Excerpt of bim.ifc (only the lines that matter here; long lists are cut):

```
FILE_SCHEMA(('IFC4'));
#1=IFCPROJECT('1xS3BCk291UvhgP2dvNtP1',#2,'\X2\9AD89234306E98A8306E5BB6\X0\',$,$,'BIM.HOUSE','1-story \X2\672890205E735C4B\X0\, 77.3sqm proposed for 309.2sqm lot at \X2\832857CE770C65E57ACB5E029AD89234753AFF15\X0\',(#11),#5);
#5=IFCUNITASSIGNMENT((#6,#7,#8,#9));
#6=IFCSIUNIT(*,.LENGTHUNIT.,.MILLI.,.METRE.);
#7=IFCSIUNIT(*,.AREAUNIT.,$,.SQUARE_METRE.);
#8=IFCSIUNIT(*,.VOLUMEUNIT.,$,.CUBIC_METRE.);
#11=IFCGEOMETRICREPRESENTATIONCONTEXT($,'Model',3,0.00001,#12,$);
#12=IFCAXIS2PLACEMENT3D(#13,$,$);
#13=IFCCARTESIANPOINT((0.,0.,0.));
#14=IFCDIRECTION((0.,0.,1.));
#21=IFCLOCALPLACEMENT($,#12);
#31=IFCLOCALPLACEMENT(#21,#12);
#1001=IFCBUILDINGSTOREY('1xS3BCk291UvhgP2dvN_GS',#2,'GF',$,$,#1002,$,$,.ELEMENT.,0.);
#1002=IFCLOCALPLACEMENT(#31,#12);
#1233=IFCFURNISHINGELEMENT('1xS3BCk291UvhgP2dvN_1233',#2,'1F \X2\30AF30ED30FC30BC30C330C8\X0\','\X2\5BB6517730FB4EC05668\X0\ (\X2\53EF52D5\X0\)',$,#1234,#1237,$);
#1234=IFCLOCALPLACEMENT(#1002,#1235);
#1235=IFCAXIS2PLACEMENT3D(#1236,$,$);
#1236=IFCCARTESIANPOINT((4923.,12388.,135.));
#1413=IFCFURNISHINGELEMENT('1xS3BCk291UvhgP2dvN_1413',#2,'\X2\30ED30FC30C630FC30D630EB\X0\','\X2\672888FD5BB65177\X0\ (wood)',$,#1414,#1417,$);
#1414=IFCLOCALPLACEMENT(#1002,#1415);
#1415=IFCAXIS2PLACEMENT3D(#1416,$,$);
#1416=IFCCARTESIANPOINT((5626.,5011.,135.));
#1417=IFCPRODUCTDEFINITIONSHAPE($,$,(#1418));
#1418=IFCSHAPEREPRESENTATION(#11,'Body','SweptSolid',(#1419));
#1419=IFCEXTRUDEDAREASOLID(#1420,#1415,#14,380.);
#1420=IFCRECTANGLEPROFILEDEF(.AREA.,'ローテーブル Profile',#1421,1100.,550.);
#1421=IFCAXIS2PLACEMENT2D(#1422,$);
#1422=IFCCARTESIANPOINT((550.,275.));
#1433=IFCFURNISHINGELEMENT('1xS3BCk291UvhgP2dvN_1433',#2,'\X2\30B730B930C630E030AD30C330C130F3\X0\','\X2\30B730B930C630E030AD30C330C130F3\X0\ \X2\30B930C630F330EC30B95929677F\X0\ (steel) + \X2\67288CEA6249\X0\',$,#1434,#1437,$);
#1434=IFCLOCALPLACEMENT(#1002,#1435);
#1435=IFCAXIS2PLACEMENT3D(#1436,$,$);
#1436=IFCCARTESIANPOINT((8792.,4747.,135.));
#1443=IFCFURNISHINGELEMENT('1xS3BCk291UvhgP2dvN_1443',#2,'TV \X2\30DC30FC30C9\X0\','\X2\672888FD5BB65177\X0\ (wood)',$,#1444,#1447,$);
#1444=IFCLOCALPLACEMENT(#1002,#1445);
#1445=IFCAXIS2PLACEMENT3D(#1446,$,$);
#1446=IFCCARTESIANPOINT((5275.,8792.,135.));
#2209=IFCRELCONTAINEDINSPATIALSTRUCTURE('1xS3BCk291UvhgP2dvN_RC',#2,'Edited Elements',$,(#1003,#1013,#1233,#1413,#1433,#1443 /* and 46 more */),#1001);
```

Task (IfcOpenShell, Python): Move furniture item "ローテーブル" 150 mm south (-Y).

```python
import ifcopenshell
import ifcopenshell.api.geometry
import ifcopenshell.util.placement
import ifcopenshell.util.unit

model = ifcopenshell.open("bim.ifc")
unit_scale = ifcopenshell.util.unit.calculate_unit_scale(model)

item = model.by_guid("1xS3BCk291UvhgP2dvN_1413")
matrix = ifcopenshell.util.placement.get_local_placement(item.ObjectPlacement)
matrix[1, 3] -= 0.15 / unit_scale
ifcopenshell.api.geometry.edit_object_placement(model, product=item, matrix=matrix, is_si=False)

print(ifcopenshell.util.placement.get_local_placement(item.ObjectPlacement).round(3) + 0.0)

model.write("bim_edited.ifc")
```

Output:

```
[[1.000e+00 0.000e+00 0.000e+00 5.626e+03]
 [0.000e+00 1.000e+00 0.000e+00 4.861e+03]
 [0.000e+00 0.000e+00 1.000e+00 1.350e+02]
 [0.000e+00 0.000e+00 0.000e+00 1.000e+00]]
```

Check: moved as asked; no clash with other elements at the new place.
